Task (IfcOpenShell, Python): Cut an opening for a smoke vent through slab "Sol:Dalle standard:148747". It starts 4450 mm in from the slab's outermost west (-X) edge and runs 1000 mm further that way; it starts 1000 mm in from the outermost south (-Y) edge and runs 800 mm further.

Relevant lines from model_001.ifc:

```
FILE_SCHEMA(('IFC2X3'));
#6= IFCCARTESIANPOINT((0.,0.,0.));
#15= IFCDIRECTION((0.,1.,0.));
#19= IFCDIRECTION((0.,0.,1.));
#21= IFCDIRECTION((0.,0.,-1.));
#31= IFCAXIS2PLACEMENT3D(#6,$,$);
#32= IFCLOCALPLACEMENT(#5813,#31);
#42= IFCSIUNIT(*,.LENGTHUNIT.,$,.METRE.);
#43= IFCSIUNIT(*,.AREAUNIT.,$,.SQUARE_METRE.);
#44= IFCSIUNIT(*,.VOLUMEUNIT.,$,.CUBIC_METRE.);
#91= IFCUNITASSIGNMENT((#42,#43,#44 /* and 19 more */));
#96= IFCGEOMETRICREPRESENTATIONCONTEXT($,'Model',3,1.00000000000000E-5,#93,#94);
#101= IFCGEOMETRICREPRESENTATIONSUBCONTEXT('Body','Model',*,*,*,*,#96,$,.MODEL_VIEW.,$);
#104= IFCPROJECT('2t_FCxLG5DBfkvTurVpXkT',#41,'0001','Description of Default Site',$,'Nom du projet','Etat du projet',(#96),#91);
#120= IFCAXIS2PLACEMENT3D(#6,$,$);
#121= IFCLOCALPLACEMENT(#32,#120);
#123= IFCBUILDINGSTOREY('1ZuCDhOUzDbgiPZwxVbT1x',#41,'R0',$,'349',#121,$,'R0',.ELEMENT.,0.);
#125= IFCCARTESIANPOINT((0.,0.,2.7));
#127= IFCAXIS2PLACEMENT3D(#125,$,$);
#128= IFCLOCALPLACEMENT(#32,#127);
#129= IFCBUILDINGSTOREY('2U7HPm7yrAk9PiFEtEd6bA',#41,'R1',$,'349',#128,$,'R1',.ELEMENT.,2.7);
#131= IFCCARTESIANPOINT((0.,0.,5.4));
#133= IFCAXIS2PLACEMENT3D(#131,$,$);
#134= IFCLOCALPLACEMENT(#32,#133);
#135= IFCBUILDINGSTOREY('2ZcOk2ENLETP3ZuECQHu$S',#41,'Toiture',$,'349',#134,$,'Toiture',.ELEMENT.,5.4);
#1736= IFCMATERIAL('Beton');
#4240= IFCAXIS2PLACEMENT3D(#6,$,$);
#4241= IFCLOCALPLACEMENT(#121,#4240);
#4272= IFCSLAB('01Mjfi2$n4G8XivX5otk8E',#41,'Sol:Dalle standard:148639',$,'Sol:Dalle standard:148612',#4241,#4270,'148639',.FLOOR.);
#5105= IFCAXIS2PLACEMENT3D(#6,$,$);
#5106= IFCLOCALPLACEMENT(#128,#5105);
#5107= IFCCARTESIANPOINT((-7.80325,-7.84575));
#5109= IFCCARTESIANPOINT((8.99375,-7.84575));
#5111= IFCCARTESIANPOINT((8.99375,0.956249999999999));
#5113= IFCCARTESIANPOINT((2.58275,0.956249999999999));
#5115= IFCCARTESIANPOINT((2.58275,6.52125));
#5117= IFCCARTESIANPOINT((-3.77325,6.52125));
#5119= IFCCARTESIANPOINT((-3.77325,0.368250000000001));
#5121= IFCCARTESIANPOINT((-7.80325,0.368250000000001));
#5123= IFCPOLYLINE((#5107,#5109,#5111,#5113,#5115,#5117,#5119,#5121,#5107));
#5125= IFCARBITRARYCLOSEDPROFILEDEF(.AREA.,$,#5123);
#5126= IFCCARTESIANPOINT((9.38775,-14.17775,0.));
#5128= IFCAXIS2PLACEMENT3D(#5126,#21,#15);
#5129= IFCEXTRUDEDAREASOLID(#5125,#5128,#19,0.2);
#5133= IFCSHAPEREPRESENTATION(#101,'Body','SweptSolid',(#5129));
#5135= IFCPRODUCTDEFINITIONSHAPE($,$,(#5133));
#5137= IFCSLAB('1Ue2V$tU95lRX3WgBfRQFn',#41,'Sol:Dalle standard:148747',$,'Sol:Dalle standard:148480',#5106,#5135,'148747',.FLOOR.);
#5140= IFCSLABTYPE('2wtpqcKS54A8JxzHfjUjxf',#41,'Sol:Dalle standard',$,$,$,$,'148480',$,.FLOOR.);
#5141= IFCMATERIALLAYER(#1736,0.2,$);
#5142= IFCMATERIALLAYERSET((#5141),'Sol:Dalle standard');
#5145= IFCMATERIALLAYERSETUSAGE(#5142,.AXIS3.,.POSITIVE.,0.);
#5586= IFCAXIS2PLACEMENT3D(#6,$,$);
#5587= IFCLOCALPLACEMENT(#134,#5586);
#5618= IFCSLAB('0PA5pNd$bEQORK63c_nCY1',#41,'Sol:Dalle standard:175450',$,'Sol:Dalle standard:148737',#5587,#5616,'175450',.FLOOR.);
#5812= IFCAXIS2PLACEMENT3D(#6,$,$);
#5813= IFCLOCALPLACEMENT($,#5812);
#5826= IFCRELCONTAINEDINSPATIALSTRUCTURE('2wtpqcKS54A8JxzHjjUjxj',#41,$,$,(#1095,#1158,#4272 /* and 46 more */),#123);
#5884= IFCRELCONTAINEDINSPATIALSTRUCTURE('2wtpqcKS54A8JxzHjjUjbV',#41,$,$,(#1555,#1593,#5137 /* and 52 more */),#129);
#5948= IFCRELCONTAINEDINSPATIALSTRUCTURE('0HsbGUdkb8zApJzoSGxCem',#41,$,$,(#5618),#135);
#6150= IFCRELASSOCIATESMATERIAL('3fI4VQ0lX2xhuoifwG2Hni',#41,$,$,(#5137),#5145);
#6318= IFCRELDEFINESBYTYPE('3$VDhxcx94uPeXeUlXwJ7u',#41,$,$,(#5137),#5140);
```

```python
import numpy as np
import ifcopenshell
import ifcopenshell.api.feature
import ifcopenshell.api.geometry
import ifcopenshell.api.root
import ifcopenshell.geom
import ifcopenshell.util.placement
import ifcopenshell.util.representation
import ifcopenshell.util.shape
import ifcopenshell.util.unit

model = ifcopenshell.open("model_001.ifc")
unit_scale = ifcopenshell.util.unit.calculate_unit_scale(model)
settings = ifcopenshell.geom.settings()


def volume(element):
    """Net volume in cubic metres, openings subtracted."""
    shape = ifcopenshell.geom.create_shape(settings, element)
    return ifcopenshell.util.shape.get_volume(shape.geometry)


slab = model.by_guid("1Ue2V$tU95lRX3WgBfRQFn")
before = volume(slab)

# Extent in the slab's own axes, in metres. The edges named are its -X and -Y sides.
slab_shape = ifcopenshell.geom.create_shape(settings, slab)
vertices = ifcopenshell.util.shape.get_vertices(slab_shape.geometry)
x_min, y_min, bottom = vertices.min(axis=0)
top = vertices[:, 2].max()

opening = ifcopenshell.api.root.create_entity(model, ifc_class="IfcOpeningElement", name="Smoke vent opening")
context = ifcopenshell.util.representation.get_context(model, "Model", "Body", "MODEL_VIEW")
width, depth = 1, 0.8
outline = [(0.0, 0.0), (width, 0.0), (width, depth), (0.0, depth), (0.0, 0.0)]
# Overshoot both faces by 50 mm so the cut is clean.
shape = ifcopenshell.api.geometry.add_slab_representation(
    model, context=context, depth=top - bottom + 0.1, polyline=outline
)
ifcopenshell.api.geometry.assign_representation(model, product=opening, representation=shape)

matrix = ifcopenshell.util.placement.get_local_placement(slab.ObjectPlacement)
matrix[:, 3] = matrix @ np.append(np.array([x_min + 4.45, y_min + 1, bottom - 0.05]) / unit_scale, 1.0)
ifcopenshell.api.geometry.edit_object_placement(model, product=opening, matrix=matrix, is_si=False)
ifcopenshell.api.feature.add_feature(model, feature=opening, element=slab)

after = volume(slab)

print(f"slab volume {before:.3f} -> {after:.3f} m3")

model.write("model_001_rev.ifc")
```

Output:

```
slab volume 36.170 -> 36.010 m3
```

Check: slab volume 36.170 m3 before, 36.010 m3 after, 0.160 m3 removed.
